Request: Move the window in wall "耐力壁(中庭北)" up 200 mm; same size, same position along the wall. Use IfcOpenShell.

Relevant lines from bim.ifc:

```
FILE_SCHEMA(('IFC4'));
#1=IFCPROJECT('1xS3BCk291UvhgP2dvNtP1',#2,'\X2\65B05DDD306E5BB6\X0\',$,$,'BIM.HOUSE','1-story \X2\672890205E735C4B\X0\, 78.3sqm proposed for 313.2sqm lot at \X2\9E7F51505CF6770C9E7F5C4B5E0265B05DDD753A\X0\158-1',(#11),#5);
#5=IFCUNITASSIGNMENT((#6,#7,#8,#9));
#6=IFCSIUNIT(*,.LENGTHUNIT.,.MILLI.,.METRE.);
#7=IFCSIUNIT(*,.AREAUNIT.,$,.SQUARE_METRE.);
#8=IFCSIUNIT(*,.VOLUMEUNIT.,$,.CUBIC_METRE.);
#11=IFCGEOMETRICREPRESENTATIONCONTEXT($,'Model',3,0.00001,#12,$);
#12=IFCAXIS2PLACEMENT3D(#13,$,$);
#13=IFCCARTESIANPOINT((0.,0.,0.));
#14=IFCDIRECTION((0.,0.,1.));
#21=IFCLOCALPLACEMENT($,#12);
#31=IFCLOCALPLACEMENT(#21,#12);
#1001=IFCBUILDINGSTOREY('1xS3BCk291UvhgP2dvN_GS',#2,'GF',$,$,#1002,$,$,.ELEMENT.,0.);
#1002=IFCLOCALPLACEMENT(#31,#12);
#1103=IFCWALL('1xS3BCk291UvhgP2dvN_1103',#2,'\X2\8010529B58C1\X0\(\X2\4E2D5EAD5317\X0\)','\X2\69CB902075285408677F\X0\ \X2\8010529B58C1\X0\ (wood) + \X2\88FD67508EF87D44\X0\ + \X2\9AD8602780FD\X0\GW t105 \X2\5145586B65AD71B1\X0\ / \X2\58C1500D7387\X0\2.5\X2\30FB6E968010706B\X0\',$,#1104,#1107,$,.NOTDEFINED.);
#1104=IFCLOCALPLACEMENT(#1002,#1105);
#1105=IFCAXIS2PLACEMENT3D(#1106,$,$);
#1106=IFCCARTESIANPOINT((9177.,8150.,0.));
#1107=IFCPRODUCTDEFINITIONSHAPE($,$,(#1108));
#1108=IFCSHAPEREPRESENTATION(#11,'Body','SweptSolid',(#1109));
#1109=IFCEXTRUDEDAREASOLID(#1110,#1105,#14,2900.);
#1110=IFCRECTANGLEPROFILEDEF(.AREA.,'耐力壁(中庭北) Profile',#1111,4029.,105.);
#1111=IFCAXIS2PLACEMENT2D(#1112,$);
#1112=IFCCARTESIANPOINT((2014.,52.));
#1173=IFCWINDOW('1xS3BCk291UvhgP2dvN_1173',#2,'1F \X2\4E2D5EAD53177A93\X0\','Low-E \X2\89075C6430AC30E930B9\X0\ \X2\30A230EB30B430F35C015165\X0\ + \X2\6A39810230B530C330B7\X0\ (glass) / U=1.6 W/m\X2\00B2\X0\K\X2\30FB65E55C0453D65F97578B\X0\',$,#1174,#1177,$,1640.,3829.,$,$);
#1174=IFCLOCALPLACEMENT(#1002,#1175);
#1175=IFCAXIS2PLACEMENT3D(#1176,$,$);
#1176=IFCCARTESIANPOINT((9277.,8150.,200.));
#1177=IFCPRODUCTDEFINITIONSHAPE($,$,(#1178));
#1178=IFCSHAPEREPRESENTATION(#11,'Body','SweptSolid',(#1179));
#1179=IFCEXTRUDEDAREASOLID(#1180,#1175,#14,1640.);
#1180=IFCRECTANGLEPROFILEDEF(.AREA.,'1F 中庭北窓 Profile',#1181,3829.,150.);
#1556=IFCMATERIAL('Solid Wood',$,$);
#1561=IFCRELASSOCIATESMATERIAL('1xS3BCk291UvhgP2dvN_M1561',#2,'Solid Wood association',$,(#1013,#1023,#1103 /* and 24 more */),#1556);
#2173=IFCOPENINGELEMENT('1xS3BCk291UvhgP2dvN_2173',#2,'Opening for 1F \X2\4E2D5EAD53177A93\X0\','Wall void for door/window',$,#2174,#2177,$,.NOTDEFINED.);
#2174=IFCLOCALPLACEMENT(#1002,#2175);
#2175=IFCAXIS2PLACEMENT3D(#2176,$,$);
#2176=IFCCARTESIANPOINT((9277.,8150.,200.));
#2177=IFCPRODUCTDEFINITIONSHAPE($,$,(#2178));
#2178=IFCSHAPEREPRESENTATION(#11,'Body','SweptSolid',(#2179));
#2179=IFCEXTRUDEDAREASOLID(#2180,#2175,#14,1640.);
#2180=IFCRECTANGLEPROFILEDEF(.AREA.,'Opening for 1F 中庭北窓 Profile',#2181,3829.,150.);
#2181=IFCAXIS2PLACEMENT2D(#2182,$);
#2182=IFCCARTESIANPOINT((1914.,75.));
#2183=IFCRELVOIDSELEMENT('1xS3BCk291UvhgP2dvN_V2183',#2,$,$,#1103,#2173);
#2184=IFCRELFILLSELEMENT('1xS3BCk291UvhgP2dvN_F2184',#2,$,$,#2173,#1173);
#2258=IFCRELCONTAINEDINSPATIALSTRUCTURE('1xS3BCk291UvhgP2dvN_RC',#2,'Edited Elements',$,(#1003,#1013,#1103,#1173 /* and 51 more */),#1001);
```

```python
import numpy as np
import ifcopenshell
import ifcopenshell.api.geometry
import ifcopenshell.util.placement
import ifcopenshell.util.unit

model = ifcopenshell.open("bim.ifc")
unit_scale = ifcopenshell.util.unit.calculate_unit_scale(model)

window = model.by_guid("1xS3BCk291UvhgP2dvN_1173")
opening = window.FillsVoids[0].RelatingOpeningElement
dz = 0.2 / unit_scale

shift = np.array([0.0, 0.0, dz])
# The window is not placed relative to its opening, so move both.
for product in (opening, window):
    matrix = ifcopenshell.util.placement.get_local_placement(product.ObjectPlacement)
    matrix[:3, 3] += shift
    ifcopenshell.api.geometry.edit_object_placement(model, product=product, matrix=matrix, is_si=False)

print(f"moved by {dz * unit_scale:+.3f} m")

model.write("bim_v2.ifc")
```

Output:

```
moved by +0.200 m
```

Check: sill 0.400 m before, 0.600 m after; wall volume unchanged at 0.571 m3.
